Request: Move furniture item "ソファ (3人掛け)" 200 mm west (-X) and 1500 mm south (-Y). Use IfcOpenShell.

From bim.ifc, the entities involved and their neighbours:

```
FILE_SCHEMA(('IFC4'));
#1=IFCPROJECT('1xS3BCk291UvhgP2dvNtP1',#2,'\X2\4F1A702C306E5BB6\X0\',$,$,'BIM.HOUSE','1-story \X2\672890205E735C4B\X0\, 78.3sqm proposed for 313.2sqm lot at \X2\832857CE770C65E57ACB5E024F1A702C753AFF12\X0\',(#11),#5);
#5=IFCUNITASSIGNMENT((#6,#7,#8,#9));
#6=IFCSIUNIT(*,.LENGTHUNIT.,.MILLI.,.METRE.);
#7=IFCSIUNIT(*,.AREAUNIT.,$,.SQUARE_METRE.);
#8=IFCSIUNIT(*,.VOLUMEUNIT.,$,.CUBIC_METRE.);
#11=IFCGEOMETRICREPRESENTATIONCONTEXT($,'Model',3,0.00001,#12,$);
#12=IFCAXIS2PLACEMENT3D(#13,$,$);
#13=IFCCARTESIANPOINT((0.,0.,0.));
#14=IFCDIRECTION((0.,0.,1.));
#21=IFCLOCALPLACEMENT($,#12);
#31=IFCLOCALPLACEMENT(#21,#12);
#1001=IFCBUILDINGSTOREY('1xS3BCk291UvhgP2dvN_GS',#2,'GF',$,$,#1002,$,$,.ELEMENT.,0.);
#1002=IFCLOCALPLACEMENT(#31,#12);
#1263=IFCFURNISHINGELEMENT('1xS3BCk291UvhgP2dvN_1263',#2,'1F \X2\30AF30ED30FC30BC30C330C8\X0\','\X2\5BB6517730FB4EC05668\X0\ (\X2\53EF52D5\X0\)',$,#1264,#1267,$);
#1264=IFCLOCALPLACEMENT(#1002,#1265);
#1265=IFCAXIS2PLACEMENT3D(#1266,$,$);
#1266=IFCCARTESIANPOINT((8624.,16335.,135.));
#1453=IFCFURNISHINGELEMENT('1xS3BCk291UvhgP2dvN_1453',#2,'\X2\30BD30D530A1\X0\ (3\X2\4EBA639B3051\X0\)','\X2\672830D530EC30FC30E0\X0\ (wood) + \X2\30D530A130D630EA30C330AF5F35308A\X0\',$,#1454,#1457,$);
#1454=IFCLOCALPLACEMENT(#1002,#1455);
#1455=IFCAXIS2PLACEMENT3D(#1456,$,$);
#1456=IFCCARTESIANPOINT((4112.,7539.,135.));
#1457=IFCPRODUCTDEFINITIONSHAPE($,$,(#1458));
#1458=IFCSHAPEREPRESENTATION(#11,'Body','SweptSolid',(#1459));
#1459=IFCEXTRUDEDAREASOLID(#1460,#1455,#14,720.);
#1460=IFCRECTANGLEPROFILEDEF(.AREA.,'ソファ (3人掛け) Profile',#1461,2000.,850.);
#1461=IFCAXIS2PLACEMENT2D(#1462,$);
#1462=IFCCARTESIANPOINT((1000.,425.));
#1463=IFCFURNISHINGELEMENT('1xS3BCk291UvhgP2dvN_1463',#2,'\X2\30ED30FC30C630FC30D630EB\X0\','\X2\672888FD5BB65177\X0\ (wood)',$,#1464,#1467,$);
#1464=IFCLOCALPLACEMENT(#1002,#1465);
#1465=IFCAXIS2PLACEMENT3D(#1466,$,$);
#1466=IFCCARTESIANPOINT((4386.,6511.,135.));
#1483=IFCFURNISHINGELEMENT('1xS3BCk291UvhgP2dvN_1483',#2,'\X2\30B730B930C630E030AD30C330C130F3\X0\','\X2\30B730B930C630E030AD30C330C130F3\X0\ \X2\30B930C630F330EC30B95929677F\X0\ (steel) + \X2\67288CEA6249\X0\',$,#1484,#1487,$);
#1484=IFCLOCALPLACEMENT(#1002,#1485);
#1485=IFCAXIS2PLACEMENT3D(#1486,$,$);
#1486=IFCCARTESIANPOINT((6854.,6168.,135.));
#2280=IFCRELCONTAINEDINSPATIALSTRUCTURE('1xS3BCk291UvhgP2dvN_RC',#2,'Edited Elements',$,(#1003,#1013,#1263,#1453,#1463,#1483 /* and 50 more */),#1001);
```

```python
import ifcopenshell
import ifcopenshell.api.geometry
import ifcopenshell.util.placement
import ifcopenshell.util.unit

model = ifcopenshell.open("bim.ifc")
unit_scale = ifcopenshell.util.unit.calculate_unit_scale(model)

item = model.by_guid("1xS3BCk291UvhgP2dvN_1453")
matrix = ifcopenshell.util.placement.get_local_placement(item.ObjectPlacement)
matrix[0, 3] -= 0.2 / unit_scale
matrix[1, 3] -= 1.5 / unit_scale
ifcopenshell.api.geometry.edit_object_placement(model, product=item, matrix=matrix, is_si=False)

print(ifcopenshell.util.placement.get_local_placement(item.ObjectPlacement).round(3) + 0.0)

model.write("bim_updated.ifc")
```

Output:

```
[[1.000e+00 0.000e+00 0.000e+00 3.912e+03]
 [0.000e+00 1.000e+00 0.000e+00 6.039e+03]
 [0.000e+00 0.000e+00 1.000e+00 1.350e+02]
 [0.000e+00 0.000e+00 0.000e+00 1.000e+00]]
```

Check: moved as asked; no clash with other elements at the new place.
